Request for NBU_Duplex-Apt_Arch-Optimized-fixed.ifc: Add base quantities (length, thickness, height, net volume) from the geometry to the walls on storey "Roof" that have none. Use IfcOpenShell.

First a look at what the model holds.

```python
import ifcopenshell
import ifcopenshell.util.element
import ifcopenshell.util.unit

model = ifcopenshell.open("NBU_Duplex-Apt_Arch-Optimized-fixed.ifc")
print(model.schema)
for unit_type in ("LENGTHUNIT", "AREAUNIT", "VOLUMEUNIT"):
    print(unit_type, ifcopenshell.util.unit.calculate_unit_scale(model, unit_type))
storey = next(s for s in model.by_type("IfcBuildingStorey") if s.Name == "Roof")
walls = [e for e in ifcopenshell.util.element.get_decomposition(storey) if e.is_a("IfcWall")]
for e in sorted(walls, key=lambda e: e.id()):
    print(e.id(), e.is_a(), e.Name, list(ifcopenshell.util.element.get_psets(e, qtos_only=True)), sep=" | ")
```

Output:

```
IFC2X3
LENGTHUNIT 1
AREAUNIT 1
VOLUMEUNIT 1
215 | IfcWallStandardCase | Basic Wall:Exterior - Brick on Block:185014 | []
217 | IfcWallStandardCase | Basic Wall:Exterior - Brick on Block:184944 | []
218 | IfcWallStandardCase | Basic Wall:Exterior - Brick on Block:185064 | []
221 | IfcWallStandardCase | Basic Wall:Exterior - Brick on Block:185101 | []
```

```python
import ifcopenshell
import ifcopenshell.api.pset
import ifcopenshell.geom
import ifcopenshell.util.element
import ifcopenshell.util.shape
import ifcopenshell.util.unit

model = ifcopenshell.open("NBU_Duplex-Apt_Arch-Optimized-fixed.ifc")
unit_scale = ifcopenshell.util.unit.calculate_unit_scale(model)
volume_scale = ifcopenshell.util.unit.calculate_unit_scale(model, "VOLUMEUNIT")
settings = ifcopenshell.geom.settings()

storey = next(s for s in model.by_type("IfcBuildingStorey") if s.Name == "Roof")
walls = [e for e in ifcopenshell.util.element.get_decomposition(storey) if e.is_a("IfcWall")]

for e in sorted(walls, key=lambda e: e.id()):
    if ifcopenshell.util.element.get_psets(e, qtos_only=True, should_inherit=False):
        continue
    # Geometry comes back in metres, in the element's own axes.
    shape = ifcopenshell.geom.create_shape(settings, e)
    values = {
        "Length": ifcopenshell.util.shape.get_x(shape.geometry) / unit_scale,
        "Width": ifcopenshell.util.shape.get_y(shape.geometry) / unit_scale,
        "Height": ifcopenshell.util.shape.get_z(shape.geometry) / unit_scale,
        "NetVolume": ifcopenshell.util.shape.get_volume(shape.geometry) / volume_scale,
    }
    qto = ifcopenshell.api.pset.add_qto(model, product=e, name="BaseQuantities")
    ifcopenshell.api.pset.edit_qto(model, qto=qto, properties=values)
    print(e.id(), {k: round(v, 3) for k, v in values.items()})

model.write("NBU_Duplex-Apt_Arch-Optimized-fixed_updated.ifc")
```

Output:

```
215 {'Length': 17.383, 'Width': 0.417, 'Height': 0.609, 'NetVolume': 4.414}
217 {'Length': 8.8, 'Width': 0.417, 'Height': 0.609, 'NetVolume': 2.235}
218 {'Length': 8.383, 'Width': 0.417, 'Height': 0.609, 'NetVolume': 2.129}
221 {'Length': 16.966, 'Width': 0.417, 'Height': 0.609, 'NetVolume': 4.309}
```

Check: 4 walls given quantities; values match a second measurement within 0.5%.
